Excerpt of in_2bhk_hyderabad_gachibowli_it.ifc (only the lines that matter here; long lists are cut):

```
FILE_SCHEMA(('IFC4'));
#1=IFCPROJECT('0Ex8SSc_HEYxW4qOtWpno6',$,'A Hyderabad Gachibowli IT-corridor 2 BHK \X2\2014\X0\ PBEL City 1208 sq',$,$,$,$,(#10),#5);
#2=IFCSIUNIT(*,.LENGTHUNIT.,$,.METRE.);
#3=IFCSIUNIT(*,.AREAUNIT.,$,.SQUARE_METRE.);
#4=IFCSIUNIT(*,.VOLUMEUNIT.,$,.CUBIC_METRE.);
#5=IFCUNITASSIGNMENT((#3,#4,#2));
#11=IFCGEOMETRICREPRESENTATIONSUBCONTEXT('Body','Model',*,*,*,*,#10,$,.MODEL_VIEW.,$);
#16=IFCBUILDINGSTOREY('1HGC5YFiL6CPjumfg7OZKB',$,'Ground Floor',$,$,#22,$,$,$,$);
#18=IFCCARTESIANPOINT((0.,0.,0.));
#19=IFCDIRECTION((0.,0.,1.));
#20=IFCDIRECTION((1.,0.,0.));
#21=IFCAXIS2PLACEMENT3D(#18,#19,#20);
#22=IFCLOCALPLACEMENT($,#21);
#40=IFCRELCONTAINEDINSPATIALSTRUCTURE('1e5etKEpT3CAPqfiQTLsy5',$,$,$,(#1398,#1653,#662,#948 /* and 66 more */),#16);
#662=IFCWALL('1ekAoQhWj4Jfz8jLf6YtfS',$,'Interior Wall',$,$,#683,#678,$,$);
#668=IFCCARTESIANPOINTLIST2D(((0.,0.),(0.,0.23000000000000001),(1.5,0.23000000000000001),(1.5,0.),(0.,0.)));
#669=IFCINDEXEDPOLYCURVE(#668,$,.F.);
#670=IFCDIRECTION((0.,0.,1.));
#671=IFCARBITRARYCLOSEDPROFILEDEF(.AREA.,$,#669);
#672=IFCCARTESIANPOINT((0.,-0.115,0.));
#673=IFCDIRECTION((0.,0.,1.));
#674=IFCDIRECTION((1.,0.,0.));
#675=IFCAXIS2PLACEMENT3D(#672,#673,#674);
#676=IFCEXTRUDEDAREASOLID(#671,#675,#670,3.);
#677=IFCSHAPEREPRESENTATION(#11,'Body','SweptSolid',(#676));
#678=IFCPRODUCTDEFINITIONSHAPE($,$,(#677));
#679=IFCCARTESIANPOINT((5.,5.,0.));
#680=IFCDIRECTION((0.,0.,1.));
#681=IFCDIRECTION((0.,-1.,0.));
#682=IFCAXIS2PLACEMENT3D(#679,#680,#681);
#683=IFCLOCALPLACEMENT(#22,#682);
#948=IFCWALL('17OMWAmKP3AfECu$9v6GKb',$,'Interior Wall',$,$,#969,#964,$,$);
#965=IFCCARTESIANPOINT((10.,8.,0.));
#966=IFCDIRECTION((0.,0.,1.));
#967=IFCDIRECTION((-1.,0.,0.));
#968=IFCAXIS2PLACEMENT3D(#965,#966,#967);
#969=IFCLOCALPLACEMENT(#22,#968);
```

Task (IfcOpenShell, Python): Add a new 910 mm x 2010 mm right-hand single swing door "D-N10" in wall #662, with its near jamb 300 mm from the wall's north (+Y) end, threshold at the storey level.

```python
import numpy as np
import ifcopenshell
import ifcopenshell.api.feature
import ifcopenshell.api.geometry
import ifcopenshell.api.root
import ifcopenshell.api.spatial
import ifcopenshell.geom
import ifcopenshell.util.element
import ifcopenshell.util.placement
import ifcopenshell.util.representation
import ifcopenshell.util.shape
import ifcopenshell.util.unit

model = ifcopenshell.open("in_2bhk_hyderabad_gachibowli_it.ifc")
unit_scale = ifcopenshell.util.unit.calculate_unit_scale(model)
settings = ifcopenshell.geom.settings()


def volume(element):
    """Net volume in cubic metres, openings subtracted."""
    shape = ifcopenshell.geom.create_shape(settings, element)
    return ifcopenshell.util.shape.get_volume(shape.geometry)


wall = model.by_guid("1ekAoQhWj4Jfz8jLf6YtfS")
storey = ifcopenshell.util.element.get_container(wall, ifc_class="IfcBuildingStorey")
context = ifcopenshell.util.representation.get_context(model, "Model", "Body", "MODEL_VIEW")
before = volume(wall)

width, height, from_end, sill = 0.91, 2.01, 0.3, 0.0  # metres

# The wall runs along its own X axis, and the end named is its -X end.
wall_shape = ifcopenshell.geom.create_shape(settings, wall)
x, y, z = ifcopenshell.util.shape.get_vertices(wall_shape.geometry).T
start = x.min() + from_end
face, thickness = float(y.min()), float(y.max() - y.min())
wall_matrix = ifcopenshell.util.placement.get_local_placement(wall.ObjectPlacement)
level = ifcopenshell.util.placement.get_local_placement(storey.ObjectPlacement)[2, 3]


def in_wall(x, y):
    """Placement at x, y metres in the wall's axes, at sill height."""
    matrix = wall_matrix.copy()
    matrix[:, 3] = wall_matrix @ np.array([x / unit_scale, y / unit_scale, 0.0, 1.0])
    matrix[2, 3] = level + sill / unit_scale
    return matrix


# Opening: a box that overshoots both wall faces by 50 mm.
opening = ifcopenshell.api.root.create_entity(model, ifc_class="IfcOpeningElement", predefined_type="OPENING")
box = ifcopenshell.api.geometry.add_wall_representation(
    model, context=context, length=width, height=height, thickness=thickness + 0.1
)
ifcopenshell.api.geometry.assign_representation(model, product=opening, representation=box)
ifcopenshell.api.geometry.edit_object_placement(model, product=opening, matrix=in_wall(start, face - 0.05), is_si=False)
ifcopenshell.api.feature.add_feature(model, feature=opening, element=wall)

door = ifcopenshell.api.root.create_entity(model, ifc_class="IfcDoor", name="D-N10", predefined_type="DOOR")
door.OverallWidth, door.OverallHeight = width / unit_scale, height / unit_scale
door.OperationType = "SINGLE_SWING_RIGHT"
body = ifcopenshell.api.geometry.add_door_representation(
    model,
    context=context,
    overall_width=door.OverallWidth,
    overall_height=door.OverallHeight,
    operation_type="SINGLE_SWING_RIGHT",
    lining_properties={"LiningDepth": thickness / unit_scale, "ThresholdDepth": thickness / unit_scale},
)
ifcopenshell.api.geometry.assign_representation(model, product=door, representation=body)
ifcopenshell.api.spatial.assign_container(model, products=[door], relating_structure=storey)
ifcopenshell.api.feature.add_filling(model, opening=opening, element=door)

# The lining spans the wall, so the door starts at the wall face.
ifcopenshell.api.geometry.edit_object_placement(model, product=door, matrix=in_wall(start, face), is_si=False)

after = volume(wall)

print(f"wall volume {before:.3f} -> {after:.3f} m3")

model.write("in_2bhk_hyderabad_gachibowli_it-out.ifc")
```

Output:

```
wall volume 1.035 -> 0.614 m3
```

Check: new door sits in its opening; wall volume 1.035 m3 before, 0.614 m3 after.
